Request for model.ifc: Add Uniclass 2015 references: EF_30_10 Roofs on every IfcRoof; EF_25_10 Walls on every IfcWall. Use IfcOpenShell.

First a look at what the model holds.

```python
import ifcopenshell

model = ifcopenshell.open("model.ifc")
print(model.schema)
print("classifications:", [c.Name for c in model.by_type("IfcClassification")])
for ifc_class in ("IfcDoor", "IfcRoof", "IfcStair", "IfcWall", "IfcWindow"):
    print(ifc_class, len(model.by_type(ifc_class)))
```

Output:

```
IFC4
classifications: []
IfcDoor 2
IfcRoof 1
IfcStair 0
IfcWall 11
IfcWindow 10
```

```python
import ifcopenshell
import ifcopenshell.api.classification

model = ifcopenshell.open("model.ifc")

system = ifcopenshell.api.classification.add_classification(model, classification="Uniclass 2015")

codes = {
    "IfcRoof": ("EF_30_10", "Roofs"),
    "IfcWall": ("EF_25_10", "Walls"),
}
for ifc_class, (code, name) in codes.items():
    products = model.by_type(ifc_class)
    ifcopenshell.api.classification.add_reference(
        model, products=products, classification=system, identification=code, name=name
    )
    print(code, len(products))

model.write("model_rev.ifc")
```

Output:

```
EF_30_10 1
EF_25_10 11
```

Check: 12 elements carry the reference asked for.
